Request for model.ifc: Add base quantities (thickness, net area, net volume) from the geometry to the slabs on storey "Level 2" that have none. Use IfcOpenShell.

First a look at what the model holds.

```python
import ifcopenshell
import ifcopenshell.util.element
import ifcopenshell.util.unit

model = ifcopenshell.open("model.ifc")
print(model.schema)
for unit_type in ("LENGTHUNIT", "AREAUNIT", "VOLUMEUNIT"):
    print(unit_type, ifcopenshell.util.unit.calculate_unit_scale(model, unit_type))
storey = next(s for s in model.by_type("IfcBuildingStorey") if s.Name == "Level 2")
slabs = [e for e in ifcopenshell.util.element.get_decomposition(storey) if e.is_a("IfcSlab")]
for e in sorted(slabs, key=lambda e: e.id()):
    print(e.id(), e.is_a(), e.Name, list(ifcopenshell.util.element.get_psets(e, qtos_only=True)), sep=" | ")
```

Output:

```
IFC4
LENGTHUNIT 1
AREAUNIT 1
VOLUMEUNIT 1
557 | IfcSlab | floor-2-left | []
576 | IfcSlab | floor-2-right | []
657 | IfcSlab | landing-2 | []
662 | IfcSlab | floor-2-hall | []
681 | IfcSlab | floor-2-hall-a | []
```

```python
import ifcopenshell
import ifcopenshell.api.pset
import ifcopenshell.geom
import ifcopenshell.util.element
import ifcopenshell.util.shape
import ifcopenshell.util.unit

model = ifcopenshell.open("model.ifc")
unit_scale = ifcopenshell.util.unit.calculate_unit_scale(model)
area_scale = ifcopenshell.util.unit.calculate_unit_scale(model, "AREAUNIT")
volume_scale = ifcopenshell.util.unit.calculate_unit_scale(model, "VOLUMEUNIT")
settings = ifcopenshell.geom.settings()

storey = next(s for s in model.by_type("IfcBuildingStorey") if s.Name == "Level 2")
slabs = [e for e in ifcopenshell.util.element.get_decomposition(storey) if e.is_a("IfcSlab")]

for e in sorted(slabs, key=lambda e: e.id()):
    if ifcopenshell.util.element.get_psets(e, qtos_only=True, should_inherit=False):
        continue
    # Geometry comes back in metres, in the element's own axes.
    shape = ifcopenshell.geom.create_shape(settings, e)
    values = {
        "Width": ifcopenshell.util.shape.get_z(shape.geometry) / unit_scale,
        "NetArea": ifcopenshell.util.shape.get_footprint_area(shape.geometry) / area_scale,
        "NetVolume": ifcopenshell.util.shape.get_volume(shape.geometry) / volume_scale,
    }
    qto = ifcopenshell.api.pset.add_qto(model, product=e, name="Qto_SlabBaseQuantities")
    ifcopenshell.api.pset.edit_qto(model, qto=qto, properties=values)
    print(e.id(), {k: round(v, 3) for k, v in values.items()})

model.write("model_rev.ifc")
```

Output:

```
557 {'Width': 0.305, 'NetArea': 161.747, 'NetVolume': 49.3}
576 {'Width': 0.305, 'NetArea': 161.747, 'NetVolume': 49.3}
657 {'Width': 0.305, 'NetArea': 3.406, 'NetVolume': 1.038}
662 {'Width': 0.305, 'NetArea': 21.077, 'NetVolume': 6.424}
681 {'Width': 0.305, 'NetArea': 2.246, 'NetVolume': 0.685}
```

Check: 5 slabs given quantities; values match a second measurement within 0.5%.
